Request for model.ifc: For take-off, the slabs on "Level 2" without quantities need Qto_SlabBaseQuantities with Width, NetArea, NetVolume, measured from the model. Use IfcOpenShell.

First a look at what the model holds.

```python
import ifcopenshell
import ifcopenshell.util.element
import ifcopenshell.util.unit

model = ifcopenshell.open("model.ifc")
print(model.schema)
for unit_type in ("LENGTHUNIT", "AREAUNIT", "VOLUMEUNIT"):
    print(unit_type, ifcopenshell.util.unit.calculate_unit_scale(model, unit_type))
storey = next(s for s in model.by_type("IfcBuildingStorey") if s.Name == "Level 2")
slabs = [e for e in ifcopenshell.util.element.get_decomposition(storey) if e.is_a("IfcSlab")]
for e in sorted(slabs, key=lambda e: e.id()):
    print(e.id(), e.is_a(), e.Name, list(ifcopenshell.util.element.get_psets(e, qtos_only=True)), sep=" | ")
```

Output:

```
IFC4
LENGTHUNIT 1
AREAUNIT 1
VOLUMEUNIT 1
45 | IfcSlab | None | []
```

```python
import ifcopenshell
import ifcopenshell.api.pset
import ifcopenshell.geom
import ifcopenshell.util.element
import ifcopenshell.util.shape
import ifcopenshell.util.unit

model = ifcopenshell.open("model.ifc")
unit_scale = ifcopenshell.util.unit.calculate_unit_scale(model)
area_scale = ifcopenshell.util.unit.calculate_unit_scale(model, "AREAUNIT")
volume_scale = ifcopenshell.util.unit.calculate_unit_scale(model, "VOLUMEUNIT")
settings = ifcopenshell.geom.settings()

storey = next(s for s in model.by_type("IfcBuildingStorey") if s.Name == "Level 2")
slabs = [e for e in ifcopenshell.util.element.get_decomposition(storey) if e.is_a("IfcSlab")]

for e in sorted(slabs, key=lambda e: e.id()):
    if ifcopenshell.util.element.get_psets(e, qtos_only=True, should_inherit=False):
        continue
    # Geometry comes back in metres, in the element's own axes.
    shape = ifcopenshell.geom.create_shape(settings, e)
    values = {
        "Width": ifcopenshell.util.shape.get_z(shape.geometry) / unit_scale,
        "NetArea": ifcopenshell.util.shape.get_footprint_area(shape.geometry) / area_scale,
        "NetVolume": ifcopenshell.util.shape.get_volume(shape.geometry) / volume_scale,
    }
    qto = ifcopenshell.api.pset.add_qto(model, product=e, name="Qto_SlabBaseQuantities")
    ifcopenshell.api.pset.edit_qto(model, qto=qto, properties=values)
    print(e.id(), {k: round(v, 3) for k, v in values.items()})

model.write("model_updated.ifc")
```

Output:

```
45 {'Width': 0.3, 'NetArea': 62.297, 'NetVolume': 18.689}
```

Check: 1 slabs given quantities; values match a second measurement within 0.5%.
